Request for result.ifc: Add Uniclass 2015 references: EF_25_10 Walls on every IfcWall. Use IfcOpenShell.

First a look at what the model holds.

```python
import ifcopenshell

model = ifcopenshell.open("result.ifc")
print(model.schema)
print("classifications:", [c.Name for c in model.by_type("IfcClassification")])
for ifc_class in ("IfcDoor", "IfcRoof", "IfcStair", "IfcWall", "IfcWindow"):
    print(ifc_class, len(model.by_type(ifc_class)))
```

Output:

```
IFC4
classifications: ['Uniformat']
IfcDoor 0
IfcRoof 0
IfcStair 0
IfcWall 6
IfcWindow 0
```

```python
import ifcopenshell
import ifcopenshell.api.classification

model = ifcopenshell.open("result.ifc")

system = ifcopenshell.api.classification.add_classification(model, classification="Uniclass 2015")

codes = {
    "IfcWall": ("EF_25_10", "Walls"),
}
for ifc_class, (code, name) in codes.items():
    products = model.by_type(ifc_class)
    ifcopenshell.api.classification.add_reference(
        model, products=products, classification=system, identification=code, name=name
    )
    print(code, len(products))

model.write("result-out.ifc")
```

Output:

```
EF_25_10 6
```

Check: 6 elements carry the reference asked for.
